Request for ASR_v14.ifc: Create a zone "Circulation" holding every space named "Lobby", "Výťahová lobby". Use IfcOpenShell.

First a look at what the model holds.

```python
import ifcopenshell

model = ifcopenshell.open("ASR_v14.ifc")
print(model.schema)
seen = {}
for space in model.by_type("IfcSpace"):
    seen[space.LongName] = seen.get(space.LongName, 0) + 1
for name, count in sorted(seen.items(), key=str):
    print(count, "x", name)
print("zones:", [z.Name for z in model.by_type("IfcZone")][:20])
```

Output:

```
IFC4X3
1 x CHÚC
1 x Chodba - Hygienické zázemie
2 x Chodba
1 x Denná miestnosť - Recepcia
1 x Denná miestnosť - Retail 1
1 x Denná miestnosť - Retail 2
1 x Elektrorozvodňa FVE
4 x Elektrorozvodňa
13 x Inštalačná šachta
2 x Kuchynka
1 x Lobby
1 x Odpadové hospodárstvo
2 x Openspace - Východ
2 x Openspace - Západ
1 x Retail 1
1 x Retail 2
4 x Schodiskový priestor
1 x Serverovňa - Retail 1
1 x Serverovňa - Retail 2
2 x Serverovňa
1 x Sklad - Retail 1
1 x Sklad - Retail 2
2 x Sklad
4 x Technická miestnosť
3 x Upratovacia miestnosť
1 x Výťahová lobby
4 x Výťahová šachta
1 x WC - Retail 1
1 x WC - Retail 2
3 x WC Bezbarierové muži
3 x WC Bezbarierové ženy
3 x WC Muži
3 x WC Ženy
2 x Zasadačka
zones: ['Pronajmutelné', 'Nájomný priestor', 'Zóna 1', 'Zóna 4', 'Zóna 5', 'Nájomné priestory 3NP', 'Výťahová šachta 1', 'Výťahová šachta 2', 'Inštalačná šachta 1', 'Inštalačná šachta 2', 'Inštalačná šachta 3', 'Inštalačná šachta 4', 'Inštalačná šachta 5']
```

```python
import ifcopenshell
import ifcopenshell.api.group
import ifcopenshell.api.root

model = ifcopenshell.open("ASR_v14.ifc")

names = {"Lobby", "Výťahová lobby"}
spaces = [s for s in model.by_type("IfcSpace") if s.LongName in names]

zone = ifcopenshell.api.root.create_entity(model, ifc_class="IfcZone", name="Circulation")
ifcopenshell.api.group.assign_group(model, products=spaces, group=zone)
print(len(spaces), "spaces in", zone.Name)

model.write("ASR_v14_v2.ifc")
```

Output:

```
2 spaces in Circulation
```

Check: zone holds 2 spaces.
